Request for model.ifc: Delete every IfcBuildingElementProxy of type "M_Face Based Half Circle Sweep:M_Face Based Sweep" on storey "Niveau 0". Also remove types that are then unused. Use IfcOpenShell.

First a look at what the model holds.

```python
import ifcopenshell
import ifcopenshell.util.element

model = ifcopenshell.open("model.ifc")
print(model.schema)
storey = next(s for s in model.by_type("IfcBuildingStorey") if s.Name == "Niveau 0")
proxies = [e for e in ifcopenshell.util.element.get_decomposition(storey) if e.is_a("IfcBuildingElementProxy")]
seen = {}
for e in proxies:
    element_type = ifcopenshell.util.element.get_type(e)
    name = element_type.Name if element_type not in (None, e) else None
    seen[name] = seen.get(name, 0) + 1
for name, count in sorted(seen.items(), key=str):
    print(count, "x", name)
```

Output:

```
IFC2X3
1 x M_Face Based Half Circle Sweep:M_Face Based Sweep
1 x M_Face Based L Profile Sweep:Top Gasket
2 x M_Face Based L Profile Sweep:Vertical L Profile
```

```python
import ifcopenshell
import ifcopenshell.api.root
import ifcopenshell.util.element

model = ifcopenshell.open("model.ifc")

storey = next(s for s in model.by_type("IfcBuildingStorey") if s.Name == "Niveau 0")
proxies = [e for e in ifcopenshell.util.element.get_decomposition(storey) if e.is_a("IfcBuildingElementProxy")]
targets = [e for e in proxies if (t := ifcopenshell.util.element.get_type(e)) not in (None, e) and t.Name == "M_Face Based Half Circle Sweep:M_Face Based Sweep"]
types = {ifcopenshell.util.element.get_type(e) for e in targets} - {None, *targets}

for e in targets:
    ifcopenshell.api.root.remove_product(model, product=e)
print(len(targets), "removed")

unused = [t for t in types if not ifcopenshell.util.element.get_types(t)]
for t in unused:
    ifcopenshell.api.root.remove_product(model, product=t)
print(len(unused), "unused types removed")

model.write("model-out.ifc")
```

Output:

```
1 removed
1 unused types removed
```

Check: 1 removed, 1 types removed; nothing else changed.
